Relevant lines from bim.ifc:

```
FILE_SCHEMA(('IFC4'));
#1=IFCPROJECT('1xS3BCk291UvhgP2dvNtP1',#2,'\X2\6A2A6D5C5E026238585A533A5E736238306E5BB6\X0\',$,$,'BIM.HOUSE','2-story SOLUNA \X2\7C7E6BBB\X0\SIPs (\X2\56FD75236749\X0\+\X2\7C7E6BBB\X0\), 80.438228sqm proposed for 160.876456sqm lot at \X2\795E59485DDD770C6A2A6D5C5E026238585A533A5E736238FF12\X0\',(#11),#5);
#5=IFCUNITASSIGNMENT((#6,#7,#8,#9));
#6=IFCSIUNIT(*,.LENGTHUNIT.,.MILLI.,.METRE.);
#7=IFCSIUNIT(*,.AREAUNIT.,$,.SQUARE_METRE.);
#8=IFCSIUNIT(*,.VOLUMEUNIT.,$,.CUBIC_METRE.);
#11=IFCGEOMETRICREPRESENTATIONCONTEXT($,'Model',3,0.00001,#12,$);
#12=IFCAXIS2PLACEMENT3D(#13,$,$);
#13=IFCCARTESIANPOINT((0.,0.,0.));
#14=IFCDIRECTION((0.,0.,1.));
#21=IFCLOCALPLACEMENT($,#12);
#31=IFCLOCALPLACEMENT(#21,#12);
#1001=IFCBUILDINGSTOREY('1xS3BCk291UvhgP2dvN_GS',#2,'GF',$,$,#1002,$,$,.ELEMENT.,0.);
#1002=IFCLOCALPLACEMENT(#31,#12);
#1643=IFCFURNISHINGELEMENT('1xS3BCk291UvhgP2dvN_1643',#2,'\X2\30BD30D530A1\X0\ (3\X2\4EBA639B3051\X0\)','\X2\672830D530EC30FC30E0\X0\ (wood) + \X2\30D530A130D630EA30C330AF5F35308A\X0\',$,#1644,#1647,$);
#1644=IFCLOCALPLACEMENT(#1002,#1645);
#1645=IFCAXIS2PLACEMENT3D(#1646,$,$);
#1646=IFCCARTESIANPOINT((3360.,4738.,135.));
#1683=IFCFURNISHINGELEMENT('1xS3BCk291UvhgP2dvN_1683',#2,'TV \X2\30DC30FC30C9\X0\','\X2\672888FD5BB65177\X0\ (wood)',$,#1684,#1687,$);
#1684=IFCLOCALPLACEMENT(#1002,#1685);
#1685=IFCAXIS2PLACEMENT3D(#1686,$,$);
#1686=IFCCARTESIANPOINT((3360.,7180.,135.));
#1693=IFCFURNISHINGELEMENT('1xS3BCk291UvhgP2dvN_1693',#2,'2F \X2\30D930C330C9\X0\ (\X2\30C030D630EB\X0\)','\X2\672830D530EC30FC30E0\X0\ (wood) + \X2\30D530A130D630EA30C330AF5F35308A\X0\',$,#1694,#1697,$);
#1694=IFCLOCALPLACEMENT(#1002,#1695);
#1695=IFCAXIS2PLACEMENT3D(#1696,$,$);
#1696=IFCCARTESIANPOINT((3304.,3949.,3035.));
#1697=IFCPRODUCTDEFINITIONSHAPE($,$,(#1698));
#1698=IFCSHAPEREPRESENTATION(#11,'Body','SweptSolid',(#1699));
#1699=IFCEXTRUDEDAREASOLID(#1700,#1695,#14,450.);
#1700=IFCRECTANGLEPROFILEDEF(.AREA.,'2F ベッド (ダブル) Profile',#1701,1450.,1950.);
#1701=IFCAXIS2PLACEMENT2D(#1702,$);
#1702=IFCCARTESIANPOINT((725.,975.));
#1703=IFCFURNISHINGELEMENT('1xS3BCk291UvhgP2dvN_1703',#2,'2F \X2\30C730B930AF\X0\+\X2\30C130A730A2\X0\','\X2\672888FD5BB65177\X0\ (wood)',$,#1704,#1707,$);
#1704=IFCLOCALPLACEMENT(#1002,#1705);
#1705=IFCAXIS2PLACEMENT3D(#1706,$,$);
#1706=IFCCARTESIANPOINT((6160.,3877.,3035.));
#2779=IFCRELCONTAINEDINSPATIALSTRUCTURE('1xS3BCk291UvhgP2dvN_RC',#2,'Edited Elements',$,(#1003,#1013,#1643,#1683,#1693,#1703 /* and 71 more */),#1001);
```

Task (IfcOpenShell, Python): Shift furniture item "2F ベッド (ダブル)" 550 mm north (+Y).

```python
import ifcopenshell
import ifcopenshell.api.geometry
import ifcopenshell.util.placement

model = ifcopenshell.open("bim.ifc")

item = model.by_id(1693)
matrix = ifcopenshell.util.placement.get_local_placement(item.ObjectPlacement)
matrix[1, 3] += 550.0
ifcopenshell.api.geometry.edit_object_placement(model, product=item, matrix=matrix, is_si=False)

print(ifcopenshell.util.placement.get_local_placement(item.ObjectPlacement).round(3) + 0.0)

model.write("bim_updated.ifc")
```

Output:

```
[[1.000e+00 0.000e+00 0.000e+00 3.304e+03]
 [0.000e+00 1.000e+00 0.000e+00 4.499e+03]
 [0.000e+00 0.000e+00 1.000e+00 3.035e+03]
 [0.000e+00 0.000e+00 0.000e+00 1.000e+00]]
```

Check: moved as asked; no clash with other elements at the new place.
